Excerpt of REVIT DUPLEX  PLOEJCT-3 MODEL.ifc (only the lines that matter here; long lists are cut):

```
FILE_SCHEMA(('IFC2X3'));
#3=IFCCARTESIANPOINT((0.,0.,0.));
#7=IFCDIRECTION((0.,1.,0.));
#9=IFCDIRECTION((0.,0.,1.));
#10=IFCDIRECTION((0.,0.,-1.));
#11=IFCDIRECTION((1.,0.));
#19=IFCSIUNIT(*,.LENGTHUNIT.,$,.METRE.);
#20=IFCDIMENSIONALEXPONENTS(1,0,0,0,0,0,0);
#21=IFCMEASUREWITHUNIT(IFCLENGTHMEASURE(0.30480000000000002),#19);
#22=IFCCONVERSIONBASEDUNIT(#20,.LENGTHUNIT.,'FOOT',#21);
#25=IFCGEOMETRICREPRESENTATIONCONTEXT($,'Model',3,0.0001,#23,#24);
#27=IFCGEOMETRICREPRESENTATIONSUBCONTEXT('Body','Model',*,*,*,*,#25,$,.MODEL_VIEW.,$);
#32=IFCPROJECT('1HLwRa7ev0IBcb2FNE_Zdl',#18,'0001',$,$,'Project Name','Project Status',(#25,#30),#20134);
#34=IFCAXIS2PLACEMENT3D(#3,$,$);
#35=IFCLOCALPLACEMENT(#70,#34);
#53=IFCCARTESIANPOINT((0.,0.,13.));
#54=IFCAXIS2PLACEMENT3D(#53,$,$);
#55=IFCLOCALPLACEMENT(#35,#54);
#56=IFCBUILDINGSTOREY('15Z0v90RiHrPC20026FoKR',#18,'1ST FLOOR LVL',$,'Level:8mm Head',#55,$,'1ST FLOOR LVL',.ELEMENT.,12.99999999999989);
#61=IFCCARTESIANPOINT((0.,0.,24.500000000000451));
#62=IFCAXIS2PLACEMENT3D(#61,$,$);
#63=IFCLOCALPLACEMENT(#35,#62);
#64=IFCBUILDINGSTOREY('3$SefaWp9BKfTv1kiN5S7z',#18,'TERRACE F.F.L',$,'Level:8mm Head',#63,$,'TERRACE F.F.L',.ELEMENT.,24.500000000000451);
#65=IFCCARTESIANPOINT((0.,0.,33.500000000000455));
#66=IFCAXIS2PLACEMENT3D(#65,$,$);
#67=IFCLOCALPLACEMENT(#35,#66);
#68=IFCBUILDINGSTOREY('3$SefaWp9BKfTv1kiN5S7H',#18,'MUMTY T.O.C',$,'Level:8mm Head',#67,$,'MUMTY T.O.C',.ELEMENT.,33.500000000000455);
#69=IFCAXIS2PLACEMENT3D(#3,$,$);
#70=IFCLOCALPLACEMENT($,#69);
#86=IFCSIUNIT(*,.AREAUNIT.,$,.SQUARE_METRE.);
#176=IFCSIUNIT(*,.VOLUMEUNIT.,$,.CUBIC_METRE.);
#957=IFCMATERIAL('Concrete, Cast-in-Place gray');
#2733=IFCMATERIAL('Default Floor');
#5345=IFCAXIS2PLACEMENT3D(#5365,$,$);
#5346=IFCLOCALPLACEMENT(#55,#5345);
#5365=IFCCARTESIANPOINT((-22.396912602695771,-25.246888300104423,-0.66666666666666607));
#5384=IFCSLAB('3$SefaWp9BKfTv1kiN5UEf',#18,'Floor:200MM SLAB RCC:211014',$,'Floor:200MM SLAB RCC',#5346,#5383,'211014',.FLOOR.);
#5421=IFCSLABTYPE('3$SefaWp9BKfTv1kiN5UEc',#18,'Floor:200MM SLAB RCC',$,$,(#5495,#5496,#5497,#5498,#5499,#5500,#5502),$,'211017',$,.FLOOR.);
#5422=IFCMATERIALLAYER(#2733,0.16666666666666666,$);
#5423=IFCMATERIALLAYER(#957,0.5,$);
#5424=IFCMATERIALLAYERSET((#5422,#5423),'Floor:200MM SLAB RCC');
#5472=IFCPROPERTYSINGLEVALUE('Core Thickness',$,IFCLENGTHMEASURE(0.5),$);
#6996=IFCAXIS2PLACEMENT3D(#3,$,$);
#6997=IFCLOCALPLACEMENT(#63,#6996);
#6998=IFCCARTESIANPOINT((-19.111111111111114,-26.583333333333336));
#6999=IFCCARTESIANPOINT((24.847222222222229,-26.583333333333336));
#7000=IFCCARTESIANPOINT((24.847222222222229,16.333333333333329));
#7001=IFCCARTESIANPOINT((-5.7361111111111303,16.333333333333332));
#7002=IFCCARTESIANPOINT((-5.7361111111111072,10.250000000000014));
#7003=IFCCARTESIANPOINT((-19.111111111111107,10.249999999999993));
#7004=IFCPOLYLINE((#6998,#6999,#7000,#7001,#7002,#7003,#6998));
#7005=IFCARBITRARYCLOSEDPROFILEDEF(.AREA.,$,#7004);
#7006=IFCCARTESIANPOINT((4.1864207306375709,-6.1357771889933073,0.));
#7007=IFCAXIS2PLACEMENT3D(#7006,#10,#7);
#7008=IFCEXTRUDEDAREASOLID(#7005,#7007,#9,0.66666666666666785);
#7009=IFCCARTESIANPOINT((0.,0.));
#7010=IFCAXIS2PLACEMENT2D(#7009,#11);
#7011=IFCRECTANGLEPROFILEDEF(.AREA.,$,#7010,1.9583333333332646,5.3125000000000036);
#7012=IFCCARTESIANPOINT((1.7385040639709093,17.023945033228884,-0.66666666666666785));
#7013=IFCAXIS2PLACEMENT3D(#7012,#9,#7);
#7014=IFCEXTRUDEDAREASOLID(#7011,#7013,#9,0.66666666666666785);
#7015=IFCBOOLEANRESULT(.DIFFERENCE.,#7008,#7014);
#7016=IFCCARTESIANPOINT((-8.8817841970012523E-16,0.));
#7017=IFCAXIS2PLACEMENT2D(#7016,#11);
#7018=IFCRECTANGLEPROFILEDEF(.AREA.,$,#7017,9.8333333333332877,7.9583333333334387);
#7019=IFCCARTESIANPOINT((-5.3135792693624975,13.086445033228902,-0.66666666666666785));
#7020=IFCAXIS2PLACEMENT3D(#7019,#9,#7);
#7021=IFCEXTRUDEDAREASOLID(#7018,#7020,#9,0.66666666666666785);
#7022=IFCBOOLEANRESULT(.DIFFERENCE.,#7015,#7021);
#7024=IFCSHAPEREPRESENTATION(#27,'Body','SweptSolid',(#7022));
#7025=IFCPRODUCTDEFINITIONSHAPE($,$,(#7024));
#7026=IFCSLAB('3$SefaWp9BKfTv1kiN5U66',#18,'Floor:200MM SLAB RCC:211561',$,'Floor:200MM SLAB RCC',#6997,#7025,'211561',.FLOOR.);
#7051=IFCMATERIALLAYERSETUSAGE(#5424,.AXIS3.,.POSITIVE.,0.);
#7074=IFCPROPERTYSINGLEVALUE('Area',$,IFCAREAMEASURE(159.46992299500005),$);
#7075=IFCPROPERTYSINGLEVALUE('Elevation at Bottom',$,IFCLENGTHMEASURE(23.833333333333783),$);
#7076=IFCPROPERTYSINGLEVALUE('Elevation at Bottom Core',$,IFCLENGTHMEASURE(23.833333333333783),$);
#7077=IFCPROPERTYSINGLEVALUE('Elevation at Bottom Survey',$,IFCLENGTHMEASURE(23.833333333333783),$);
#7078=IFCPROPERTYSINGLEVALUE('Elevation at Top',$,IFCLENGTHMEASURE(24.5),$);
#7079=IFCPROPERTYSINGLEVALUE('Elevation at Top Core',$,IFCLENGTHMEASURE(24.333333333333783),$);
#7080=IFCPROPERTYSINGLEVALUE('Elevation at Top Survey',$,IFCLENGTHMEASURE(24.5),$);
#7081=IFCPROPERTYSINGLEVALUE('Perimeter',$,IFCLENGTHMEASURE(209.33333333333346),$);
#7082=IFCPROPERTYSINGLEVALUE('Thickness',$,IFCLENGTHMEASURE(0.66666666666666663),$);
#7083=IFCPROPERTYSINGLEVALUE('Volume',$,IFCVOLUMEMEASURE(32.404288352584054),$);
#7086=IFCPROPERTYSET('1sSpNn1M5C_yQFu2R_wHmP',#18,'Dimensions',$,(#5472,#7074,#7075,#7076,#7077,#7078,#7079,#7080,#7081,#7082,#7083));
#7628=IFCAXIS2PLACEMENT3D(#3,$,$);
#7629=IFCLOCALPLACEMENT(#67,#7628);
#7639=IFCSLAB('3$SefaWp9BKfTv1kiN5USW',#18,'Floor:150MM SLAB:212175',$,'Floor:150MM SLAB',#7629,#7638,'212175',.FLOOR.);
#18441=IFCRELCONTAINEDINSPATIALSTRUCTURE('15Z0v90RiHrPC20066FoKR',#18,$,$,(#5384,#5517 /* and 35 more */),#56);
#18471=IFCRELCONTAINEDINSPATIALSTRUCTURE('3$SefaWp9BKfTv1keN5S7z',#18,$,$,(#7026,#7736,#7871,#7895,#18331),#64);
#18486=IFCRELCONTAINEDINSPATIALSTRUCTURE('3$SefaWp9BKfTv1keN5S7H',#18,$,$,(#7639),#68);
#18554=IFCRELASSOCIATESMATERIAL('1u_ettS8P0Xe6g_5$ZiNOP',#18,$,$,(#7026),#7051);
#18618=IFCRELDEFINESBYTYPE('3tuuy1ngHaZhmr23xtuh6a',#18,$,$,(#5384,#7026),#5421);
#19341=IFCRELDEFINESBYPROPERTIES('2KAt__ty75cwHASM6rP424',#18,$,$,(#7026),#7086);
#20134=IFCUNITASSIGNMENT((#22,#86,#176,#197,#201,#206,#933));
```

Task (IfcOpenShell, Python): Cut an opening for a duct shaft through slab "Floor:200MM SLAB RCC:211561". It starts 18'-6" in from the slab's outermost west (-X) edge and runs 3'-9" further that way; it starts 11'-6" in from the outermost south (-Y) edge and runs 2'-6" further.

```python
import numpy as np
import ifcopenshell
import ifcopenshell.api.feature
import ifcopenshell.api.geometry
import ifcopenshell.api.pset
import ifcopenshell.api.root
import ifcopenshell.geom
import ifcopenshell.util.element
import ifcopenshell.util.placement
import ifcopenshell.util.representation
import ifcopenshell.util.shape
import ifcopenshell.util.unit

model = ifcopenshell.open("REVIT DUPLEX  PLOEJCT-3 MODEL.ifc")
unit_scale = ifcopenshell.util.unit.calculate_unit_scale(model)
area_scale = ifcopenshell.util.unit.calculate_unit_scale(model, "AREAUNIT")
volume_scale = ifcopenshell.util.unit.calculate_unit_scale(model, "VOLUMEUNIT")
settings = ifcopenshell.geom.settings()


def volume(element):
    """Net volume in cubic metres, openings subtracted."""
    shape = ifcopenshell.geom.create_shape(settings, element)
    return ifcopenshell.util.shape.get_volume(shape.geometry)


slab = model.by_id(7026)
before = volume(slab)

# Extent in the slab's own axes, in metres. The edges named are its -X and -Y sides.
slab_shape = ifcopenshell.geom.create_shape(settings, slab)
vertices = ifcopenshell.util.shape.get_vertices(slab_shape.geometry)
x_min, y_min, bottom = vertices.min(axis=0)
top = vertices[:, 2].max()

opening = ifcopenshell.api.root.create_entity(model, ifc_class="IfcOpeningElement", name="Duct shaft opening")
context = ifcopenshell.util.representation.get_context(model, "Model", "Body", "MODEL_VIEW")
width, depth = 1.143, 0.762
outline = [(0.0, 0.0), (width, 0.0), (width, depth), (0.0, depth), (0.0, 0.0)]
# Overshoot both faces by 50 mm so the cut is clean.
shape = ifcopenshell.api.geometry.add_slab_representation(
    model, context=context, depth=top - bottom + 0.1, polyline=outline
)
ifcopenshell.api.geometry.assign_representation(model, product=opening, representation=shape)

matrix = ifcopenshell.util.placement.get_local_placement(slab.ObjectPlacement)
matrix[:, 3] = matrix @ np.append(np.array([x_min + 5.6388, y_min + 3.5052, bottom - 0.05]) / unit_scale, 1.0)
ifcopenshell.api.geometry.edit_object_placement(model, product=opening, matrix=matrix, is_si=False)
ifcopenshell.api.feature.add_feature(model, feature=opening, element=slab)

after = volume(slab)

# Update the slab's stored quantities.
pset = model.by_id(ifcopenshell.util.element.get_pset(slab, "Dimensions", should_inherit=False)["id"])
ifcopenshell.api.pset.edit_pset(model, pset=pset, properties={
    "Area": model.create_entity("IfcAreaMeasure", after / (top - bottom) / area_scale),
    "Volume": model.create_entity("IfcVolumeMeasure", after / volume_scale),
})

print(f"slab volume {before:.3f} -> {after:.3f} m3")

model.write("REVIT DUPLEX  PLOEJCT-3 MODEL_updated.ifc")
```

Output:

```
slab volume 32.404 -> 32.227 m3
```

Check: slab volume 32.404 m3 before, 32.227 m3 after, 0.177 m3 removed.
